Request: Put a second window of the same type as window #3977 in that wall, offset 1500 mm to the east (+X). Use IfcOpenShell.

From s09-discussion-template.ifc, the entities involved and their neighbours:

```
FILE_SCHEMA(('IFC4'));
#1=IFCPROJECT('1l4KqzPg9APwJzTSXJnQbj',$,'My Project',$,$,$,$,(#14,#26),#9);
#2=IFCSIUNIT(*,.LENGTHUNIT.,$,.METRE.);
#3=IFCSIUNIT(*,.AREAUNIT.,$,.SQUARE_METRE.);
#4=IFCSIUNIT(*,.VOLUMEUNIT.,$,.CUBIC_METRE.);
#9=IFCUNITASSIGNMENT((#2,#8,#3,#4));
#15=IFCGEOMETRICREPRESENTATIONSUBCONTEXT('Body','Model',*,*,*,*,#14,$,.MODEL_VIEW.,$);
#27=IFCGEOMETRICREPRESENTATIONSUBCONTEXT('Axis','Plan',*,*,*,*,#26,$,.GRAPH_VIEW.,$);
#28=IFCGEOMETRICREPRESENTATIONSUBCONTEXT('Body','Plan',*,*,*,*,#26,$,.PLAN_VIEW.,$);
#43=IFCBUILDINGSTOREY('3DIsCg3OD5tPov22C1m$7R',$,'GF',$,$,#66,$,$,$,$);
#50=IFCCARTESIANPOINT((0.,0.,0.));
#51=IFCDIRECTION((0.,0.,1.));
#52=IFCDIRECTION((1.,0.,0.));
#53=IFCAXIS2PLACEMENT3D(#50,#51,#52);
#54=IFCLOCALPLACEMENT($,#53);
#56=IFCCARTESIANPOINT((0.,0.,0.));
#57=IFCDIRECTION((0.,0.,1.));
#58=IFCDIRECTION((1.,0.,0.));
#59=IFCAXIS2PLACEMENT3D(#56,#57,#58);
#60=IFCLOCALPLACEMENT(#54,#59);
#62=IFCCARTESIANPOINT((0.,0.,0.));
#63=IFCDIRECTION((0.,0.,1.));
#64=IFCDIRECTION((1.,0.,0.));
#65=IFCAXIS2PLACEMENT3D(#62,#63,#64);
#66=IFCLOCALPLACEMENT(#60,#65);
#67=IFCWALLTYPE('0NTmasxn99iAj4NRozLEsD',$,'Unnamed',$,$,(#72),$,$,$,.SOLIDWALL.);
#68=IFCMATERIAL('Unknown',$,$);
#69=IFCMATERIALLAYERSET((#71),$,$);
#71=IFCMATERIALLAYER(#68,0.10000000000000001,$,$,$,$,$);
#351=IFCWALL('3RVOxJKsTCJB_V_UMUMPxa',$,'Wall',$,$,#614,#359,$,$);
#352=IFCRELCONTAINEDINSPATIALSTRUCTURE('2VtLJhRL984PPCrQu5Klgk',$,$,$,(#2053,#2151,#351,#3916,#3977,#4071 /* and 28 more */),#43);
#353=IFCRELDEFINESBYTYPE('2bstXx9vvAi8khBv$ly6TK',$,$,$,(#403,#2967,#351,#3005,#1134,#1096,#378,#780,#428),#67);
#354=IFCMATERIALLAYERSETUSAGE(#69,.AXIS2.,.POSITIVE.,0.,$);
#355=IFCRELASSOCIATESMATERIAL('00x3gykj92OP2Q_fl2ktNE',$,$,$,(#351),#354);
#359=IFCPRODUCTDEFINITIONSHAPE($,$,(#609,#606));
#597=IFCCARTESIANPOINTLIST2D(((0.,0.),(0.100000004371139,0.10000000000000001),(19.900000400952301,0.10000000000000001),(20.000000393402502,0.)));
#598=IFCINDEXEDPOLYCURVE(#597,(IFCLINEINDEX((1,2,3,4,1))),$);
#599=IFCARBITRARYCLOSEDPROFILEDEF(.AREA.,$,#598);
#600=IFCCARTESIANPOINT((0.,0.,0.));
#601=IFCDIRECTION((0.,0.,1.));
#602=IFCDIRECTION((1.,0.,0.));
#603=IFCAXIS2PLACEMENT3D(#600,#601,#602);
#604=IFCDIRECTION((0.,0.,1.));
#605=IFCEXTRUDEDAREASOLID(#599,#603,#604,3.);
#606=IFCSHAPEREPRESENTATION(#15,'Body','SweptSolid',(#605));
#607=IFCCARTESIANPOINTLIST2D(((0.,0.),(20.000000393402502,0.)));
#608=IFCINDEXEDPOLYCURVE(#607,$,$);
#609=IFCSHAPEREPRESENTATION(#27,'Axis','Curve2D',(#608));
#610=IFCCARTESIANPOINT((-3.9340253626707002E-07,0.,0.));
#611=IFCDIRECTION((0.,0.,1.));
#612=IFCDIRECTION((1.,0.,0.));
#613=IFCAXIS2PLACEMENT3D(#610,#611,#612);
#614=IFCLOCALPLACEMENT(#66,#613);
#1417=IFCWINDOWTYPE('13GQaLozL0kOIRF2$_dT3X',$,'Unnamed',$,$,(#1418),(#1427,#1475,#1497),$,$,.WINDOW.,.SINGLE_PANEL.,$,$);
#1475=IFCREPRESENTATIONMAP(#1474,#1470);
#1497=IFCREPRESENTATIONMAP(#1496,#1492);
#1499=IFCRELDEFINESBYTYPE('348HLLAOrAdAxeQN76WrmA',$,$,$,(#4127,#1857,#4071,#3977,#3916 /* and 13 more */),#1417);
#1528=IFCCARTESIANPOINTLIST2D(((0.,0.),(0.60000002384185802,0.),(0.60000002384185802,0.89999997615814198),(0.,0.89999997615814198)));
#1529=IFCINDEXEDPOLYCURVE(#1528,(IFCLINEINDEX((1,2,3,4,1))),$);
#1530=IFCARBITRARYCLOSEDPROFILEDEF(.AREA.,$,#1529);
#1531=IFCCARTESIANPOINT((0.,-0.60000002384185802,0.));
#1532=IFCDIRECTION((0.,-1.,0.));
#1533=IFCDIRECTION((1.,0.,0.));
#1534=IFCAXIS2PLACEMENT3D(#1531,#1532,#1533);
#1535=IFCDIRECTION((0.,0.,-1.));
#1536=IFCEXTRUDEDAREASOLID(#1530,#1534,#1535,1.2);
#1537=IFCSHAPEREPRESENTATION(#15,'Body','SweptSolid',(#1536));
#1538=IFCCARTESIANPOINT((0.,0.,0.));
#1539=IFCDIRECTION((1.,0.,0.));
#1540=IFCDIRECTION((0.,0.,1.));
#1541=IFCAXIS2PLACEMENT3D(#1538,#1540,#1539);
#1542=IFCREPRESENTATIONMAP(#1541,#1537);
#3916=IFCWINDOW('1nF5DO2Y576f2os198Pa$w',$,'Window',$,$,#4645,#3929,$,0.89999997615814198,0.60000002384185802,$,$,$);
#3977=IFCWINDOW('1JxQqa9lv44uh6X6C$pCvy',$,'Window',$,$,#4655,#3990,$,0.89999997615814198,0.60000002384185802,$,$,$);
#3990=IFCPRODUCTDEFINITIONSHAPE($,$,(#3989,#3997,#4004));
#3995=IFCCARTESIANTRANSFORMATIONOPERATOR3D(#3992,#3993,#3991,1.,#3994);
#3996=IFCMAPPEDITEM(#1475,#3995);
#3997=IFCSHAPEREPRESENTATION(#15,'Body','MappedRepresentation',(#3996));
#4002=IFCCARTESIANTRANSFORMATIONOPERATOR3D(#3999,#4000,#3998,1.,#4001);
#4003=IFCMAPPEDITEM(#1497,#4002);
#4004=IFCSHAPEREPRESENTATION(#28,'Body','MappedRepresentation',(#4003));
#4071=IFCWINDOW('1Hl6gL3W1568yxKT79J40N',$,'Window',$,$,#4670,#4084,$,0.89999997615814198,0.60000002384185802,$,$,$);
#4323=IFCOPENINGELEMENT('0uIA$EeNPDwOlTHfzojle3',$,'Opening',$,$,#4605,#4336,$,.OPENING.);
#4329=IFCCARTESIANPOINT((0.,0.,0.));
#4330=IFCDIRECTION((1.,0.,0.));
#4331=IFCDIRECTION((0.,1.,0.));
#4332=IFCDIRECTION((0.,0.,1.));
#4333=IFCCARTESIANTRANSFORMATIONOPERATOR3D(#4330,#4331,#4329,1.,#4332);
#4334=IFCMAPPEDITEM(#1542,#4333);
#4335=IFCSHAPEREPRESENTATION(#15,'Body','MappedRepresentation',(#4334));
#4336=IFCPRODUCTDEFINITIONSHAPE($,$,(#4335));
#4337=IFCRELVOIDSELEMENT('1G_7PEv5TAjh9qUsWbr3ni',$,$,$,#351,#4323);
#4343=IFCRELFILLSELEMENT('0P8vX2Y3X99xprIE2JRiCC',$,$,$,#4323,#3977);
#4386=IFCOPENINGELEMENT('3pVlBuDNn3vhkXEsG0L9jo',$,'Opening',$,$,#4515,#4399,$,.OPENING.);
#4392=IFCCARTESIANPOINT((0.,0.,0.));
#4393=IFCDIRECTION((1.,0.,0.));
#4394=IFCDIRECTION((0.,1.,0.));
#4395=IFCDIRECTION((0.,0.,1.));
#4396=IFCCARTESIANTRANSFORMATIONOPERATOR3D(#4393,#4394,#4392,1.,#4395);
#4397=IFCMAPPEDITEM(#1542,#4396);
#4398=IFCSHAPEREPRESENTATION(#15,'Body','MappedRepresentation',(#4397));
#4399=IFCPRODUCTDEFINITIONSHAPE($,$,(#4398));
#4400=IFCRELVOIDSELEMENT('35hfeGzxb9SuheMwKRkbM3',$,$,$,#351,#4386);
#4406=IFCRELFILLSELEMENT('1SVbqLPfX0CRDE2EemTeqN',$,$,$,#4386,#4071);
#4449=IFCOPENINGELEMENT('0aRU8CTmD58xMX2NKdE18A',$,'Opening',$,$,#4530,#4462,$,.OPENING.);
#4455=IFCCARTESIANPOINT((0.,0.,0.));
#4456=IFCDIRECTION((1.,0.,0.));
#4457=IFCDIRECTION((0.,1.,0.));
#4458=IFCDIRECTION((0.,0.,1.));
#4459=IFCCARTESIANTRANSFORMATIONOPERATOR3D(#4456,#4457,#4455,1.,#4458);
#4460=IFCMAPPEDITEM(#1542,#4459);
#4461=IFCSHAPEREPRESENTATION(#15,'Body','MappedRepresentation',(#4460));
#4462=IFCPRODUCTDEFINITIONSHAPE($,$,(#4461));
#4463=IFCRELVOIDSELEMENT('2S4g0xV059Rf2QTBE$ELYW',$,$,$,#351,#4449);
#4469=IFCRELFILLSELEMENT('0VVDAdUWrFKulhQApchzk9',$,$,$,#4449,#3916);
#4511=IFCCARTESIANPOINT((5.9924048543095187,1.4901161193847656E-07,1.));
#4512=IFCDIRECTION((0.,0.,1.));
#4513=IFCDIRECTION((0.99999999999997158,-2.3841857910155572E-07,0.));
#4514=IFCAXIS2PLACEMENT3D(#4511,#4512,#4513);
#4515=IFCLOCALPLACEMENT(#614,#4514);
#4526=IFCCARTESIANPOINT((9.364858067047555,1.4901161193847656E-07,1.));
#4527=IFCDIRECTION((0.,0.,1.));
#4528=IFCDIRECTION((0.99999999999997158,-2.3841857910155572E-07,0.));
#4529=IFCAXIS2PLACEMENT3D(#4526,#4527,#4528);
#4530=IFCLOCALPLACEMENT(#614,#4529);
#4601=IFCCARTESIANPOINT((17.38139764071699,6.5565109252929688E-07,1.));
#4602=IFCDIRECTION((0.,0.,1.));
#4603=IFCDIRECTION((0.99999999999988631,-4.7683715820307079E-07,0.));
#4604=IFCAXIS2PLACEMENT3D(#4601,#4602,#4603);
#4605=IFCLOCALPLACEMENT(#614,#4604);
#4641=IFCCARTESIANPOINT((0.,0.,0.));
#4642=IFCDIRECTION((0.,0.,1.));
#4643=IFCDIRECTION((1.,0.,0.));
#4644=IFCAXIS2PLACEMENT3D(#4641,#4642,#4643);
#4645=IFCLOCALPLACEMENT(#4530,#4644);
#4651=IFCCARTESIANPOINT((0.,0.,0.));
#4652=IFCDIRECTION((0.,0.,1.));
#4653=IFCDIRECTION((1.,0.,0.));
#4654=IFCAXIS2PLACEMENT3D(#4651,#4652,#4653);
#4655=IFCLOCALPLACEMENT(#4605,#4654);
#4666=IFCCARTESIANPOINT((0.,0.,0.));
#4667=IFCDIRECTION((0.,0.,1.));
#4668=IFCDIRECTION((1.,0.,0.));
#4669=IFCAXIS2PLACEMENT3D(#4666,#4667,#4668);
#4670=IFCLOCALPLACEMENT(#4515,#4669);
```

```python
import ifcopenshell
import ifcopenshell.api.feature
import ifcopenshell.api.geometry
import ifcopenshell.api.root
import ifcopenshell.geom
import ifcopenshell.util.element
import ifcopenshell.util.placement
import ifcopenshell.util.shape

model = ifcopenshell.open("s09-discussion-template.ifc")
settings = ifcopenshell.geom.settings()


def volume(element):
    """Net volume in cubic metres, openings subtracted."""
    shape = ifcopenshell.geom.create_shape(settings, element)
    return ifcopenshell.util.shape.get_volume(shape.geometry)


window = model.by_guid("1JxQqa9lv44uh6X6C$pCvy")
opening = window.FillsVoids[0].RelatingOpeningElement
wall = opening.VoidsElements[0].RelatingBuildingElement
before = volume(wall)
shift = ifcopenshell.util.placement.get_local_placement(wall.ObjectPlacement)[:3, 0] * 1.5

# copy_class copies the void relationship, type, container and properties, but no geometry.
new_opening = ifcopenshell.api.root.copy_class(model, product=opening)
new_opening.Representation = ifcopenshell.util.element.copy_deep(
    model, opening.Representation, exclude=["IfcGeometricRepresentationContext", "IfcRepresentationMap"]
)
new_window = ifcopenshell.api.root.copy_class(model, product=window)
new_window.Representation = ifcopenshell.util.element.copy_deep(
    model, window.Representation, exclude=["IfcGeometricRepresentationContext", "IfcRepresentationMap"]
)
ifcopenshell.api.feature.add_filling(model, opening=new_opening, element=new_window)

for old, new in ((opening, new_opening), (window, new_window)):
    matrix = ifcopenshell.util.placement.get_local_placement(old.ObjectPlacement)
    matrix[:3, 3] += shift
    ifcopenshell.api.geometry.edit_object_placement(model, product=new, matrix=matrix, is_si=False)

after = volume(wall)

print(f"wall volume {before:.3f} -> {after:.3f} m3")

model.write("s09-discussion-template_rev.ifc")
```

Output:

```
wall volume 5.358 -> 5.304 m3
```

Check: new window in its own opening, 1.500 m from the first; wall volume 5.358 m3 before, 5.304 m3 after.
